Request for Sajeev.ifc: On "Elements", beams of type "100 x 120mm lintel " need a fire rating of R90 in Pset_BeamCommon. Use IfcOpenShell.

First a look at what the model holds.

```python
import ifcopenshell
import ifcopenshell.util.element

model = ifcopenshell.open("Sajeev.ifc")
print(model.schema)
storey = next(s for s in model.by_type("IfcBuildingStorey") if s.Name == "Elements")
beams = [e for e in ifcopenshell.util.element.get_decomposition(storey) if e.is_a("IfcBeam")]
seen = {}
for e in beams:
    element_type = ifcopenshell.util.element.get_type(e)
    key = (element_type.Name if element_type != e and element_type else None, ifcopenshell.util.element.get_pset(e, "Pset_BeamCommon", "FireRating"))
    seen[key] = seen.get(key, 0) + 1
for (name, value), count in sorted(seen.items(), key=str):
    print(count, "x", name, "|", value)
```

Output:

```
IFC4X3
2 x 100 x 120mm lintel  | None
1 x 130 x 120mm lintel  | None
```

```python
import ifcopenshell
import ifcopenshell.api.pset
import ifcopenshell.util.element

model = ifcopenshell.open("Sajeev.ifc")

storey = next(s for s in model.by_type("IfcBuildingStorey") if s.Name == "Elements")
beams = [e for e in ifcopenshell.util.element.get_decomposition(storey) if e.is_a("IfcBeam")]

count = 0
for e in beams:
    element_type = ifcopenshell.util.element.get_type(e)
    if element_type in (None, e) or element_type.Name != "100 x 120mm lintel ":
        continue
    # add_pset returns the element's existing set when there is one.
    pset = ifcopenshell.api.pset.add_pset(model, product=e, name="Pset_BeamCommon")
    ifcopenshell.api.pset.edit_pset(model, pset=pset, properties={"FireRating": "R90"})
    count += 1

print(count, "beams updated")

model.write("Sajeev_updated.ifc")
```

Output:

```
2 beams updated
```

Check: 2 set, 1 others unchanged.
